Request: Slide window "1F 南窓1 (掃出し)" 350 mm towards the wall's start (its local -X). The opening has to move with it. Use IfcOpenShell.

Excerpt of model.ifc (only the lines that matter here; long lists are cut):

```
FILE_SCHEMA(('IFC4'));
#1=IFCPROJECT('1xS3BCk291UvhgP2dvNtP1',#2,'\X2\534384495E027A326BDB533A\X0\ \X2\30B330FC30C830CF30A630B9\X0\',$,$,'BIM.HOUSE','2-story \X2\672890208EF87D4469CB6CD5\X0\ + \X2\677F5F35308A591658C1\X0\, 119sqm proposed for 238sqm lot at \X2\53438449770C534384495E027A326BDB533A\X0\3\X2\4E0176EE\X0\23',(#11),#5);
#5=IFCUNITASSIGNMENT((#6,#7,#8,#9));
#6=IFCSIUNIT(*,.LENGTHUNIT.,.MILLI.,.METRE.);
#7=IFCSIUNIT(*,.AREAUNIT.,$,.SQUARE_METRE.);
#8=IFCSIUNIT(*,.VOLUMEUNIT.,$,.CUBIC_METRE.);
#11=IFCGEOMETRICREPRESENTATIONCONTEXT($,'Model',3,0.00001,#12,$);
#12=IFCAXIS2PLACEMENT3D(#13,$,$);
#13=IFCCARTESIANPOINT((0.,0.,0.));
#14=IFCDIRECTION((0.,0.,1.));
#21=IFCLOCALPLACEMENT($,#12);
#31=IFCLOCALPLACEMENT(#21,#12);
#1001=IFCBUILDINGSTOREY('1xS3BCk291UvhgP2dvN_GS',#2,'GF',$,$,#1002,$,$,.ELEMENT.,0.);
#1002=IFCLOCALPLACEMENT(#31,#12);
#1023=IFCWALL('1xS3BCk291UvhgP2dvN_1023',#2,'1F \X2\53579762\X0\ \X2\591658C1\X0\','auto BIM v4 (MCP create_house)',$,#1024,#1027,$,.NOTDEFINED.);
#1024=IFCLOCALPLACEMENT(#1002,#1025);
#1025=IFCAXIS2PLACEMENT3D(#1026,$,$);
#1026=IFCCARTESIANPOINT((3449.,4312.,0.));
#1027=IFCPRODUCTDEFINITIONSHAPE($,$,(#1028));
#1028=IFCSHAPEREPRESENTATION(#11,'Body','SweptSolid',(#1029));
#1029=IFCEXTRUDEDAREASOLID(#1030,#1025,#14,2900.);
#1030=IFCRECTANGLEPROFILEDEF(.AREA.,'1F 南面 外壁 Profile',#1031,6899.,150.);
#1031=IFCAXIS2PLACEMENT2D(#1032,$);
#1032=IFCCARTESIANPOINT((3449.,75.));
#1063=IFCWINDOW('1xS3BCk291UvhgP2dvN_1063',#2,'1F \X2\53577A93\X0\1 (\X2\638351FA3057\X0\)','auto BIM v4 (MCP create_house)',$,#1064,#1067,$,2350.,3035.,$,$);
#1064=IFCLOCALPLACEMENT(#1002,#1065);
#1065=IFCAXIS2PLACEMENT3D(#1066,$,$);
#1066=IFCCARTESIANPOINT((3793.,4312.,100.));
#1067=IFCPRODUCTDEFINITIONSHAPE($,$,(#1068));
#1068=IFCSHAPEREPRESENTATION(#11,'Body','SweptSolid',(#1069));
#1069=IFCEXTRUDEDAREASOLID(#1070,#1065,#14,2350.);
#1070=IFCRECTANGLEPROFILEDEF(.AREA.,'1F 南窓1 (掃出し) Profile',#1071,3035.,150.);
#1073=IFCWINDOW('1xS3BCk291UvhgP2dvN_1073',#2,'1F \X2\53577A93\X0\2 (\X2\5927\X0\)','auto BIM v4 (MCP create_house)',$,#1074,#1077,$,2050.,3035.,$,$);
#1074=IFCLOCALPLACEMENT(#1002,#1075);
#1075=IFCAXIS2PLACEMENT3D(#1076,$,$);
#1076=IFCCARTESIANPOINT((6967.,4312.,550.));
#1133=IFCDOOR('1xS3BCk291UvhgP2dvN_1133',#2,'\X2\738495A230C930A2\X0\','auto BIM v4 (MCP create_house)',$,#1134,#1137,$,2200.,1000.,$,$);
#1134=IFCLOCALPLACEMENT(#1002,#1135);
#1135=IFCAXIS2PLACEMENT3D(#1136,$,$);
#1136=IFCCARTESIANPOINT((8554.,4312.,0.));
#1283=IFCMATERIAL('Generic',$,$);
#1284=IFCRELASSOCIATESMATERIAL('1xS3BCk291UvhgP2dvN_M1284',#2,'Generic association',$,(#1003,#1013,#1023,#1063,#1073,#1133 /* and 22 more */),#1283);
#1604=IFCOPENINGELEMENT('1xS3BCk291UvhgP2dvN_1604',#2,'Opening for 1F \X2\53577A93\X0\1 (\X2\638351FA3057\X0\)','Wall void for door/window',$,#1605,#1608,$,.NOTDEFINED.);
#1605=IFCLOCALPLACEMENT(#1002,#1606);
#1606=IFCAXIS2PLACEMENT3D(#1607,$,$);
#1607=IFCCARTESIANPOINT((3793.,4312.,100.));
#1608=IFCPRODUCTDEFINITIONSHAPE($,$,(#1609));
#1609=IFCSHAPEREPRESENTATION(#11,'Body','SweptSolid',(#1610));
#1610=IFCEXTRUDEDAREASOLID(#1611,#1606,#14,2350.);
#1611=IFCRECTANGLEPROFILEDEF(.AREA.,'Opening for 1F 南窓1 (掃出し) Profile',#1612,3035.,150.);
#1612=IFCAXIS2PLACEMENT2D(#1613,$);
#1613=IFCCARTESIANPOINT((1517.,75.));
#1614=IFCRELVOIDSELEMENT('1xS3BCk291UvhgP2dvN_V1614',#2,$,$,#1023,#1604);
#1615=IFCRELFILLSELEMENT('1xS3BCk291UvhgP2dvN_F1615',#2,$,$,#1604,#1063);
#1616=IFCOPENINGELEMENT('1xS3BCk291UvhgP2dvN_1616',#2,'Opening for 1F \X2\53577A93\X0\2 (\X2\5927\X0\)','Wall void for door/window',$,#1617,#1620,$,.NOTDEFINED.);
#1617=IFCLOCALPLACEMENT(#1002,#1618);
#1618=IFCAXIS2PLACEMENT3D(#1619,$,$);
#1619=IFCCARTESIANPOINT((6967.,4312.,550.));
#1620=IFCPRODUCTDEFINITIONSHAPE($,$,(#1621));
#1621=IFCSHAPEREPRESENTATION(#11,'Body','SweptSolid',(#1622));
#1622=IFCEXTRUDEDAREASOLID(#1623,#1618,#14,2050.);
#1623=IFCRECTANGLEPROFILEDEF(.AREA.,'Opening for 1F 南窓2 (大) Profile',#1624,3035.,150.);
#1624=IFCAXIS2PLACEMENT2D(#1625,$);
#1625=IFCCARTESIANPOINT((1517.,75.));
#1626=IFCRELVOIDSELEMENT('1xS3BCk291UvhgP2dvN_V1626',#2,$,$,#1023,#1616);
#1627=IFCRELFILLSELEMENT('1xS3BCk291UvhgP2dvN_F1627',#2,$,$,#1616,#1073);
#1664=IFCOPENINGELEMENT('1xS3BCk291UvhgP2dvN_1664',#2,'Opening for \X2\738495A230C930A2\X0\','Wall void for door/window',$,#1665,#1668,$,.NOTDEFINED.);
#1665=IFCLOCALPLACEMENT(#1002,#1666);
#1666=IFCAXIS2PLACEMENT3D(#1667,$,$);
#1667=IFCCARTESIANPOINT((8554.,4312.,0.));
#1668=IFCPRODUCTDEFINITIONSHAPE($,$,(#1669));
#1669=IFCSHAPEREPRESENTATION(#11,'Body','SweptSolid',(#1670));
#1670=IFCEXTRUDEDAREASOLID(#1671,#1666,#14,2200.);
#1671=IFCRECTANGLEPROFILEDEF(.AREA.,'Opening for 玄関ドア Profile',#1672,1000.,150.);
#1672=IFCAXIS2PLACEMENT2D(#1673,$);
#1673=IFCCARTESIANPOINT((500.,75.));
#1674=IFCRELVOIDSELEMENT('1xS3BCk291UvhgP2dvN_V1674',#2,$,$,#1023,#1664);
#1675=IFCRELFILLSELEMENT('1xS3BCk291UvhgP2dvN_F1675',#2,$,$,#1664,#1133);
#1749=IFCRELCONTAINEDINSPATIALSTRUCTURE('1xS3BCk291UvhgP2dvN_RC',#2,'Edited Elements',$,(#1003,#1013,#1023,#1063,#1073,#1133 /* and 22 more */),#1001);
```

```python
import ifcopenshell
import ifcopenshell.api.geometry
import ifcopenshell.util.placement

model = ifcopenshell.open("model.ifc")

window = model.by_id(1063)
opening = window.FillsVoids[0].RelatingOpeningElement
wall = opening.VoidsElements[0].RelatingBuildingElement

wall_matrix = ifcopenshell.util.placement.get_local_placement(wall.ObjectPlacement)
shift = wall_matrix[:3, 0] * -350.0
before = ifcopenshell.util.placement.get_local_placement(window.ObjectPlacement)[:3, 3].copy()

# The window is not placed relative to its opening, so move both.
for product in (opening, window):
    matrix = ifcopenshell.util.placement.get_local_placement(product.ObjectPlacement)
    matrix[:3, 3] += shift
    ifcopenshell.api.geometry.edit_object_placement(model, product=product, matrix=matrix, is_si=False)

after = ifcopenshell.util.placement.get_local_placement(window.ObjectPlacement)[:3, 3]
print("window moved by", (after - before).round(3) + 0.0)

model.write("model_v2.ifc")
```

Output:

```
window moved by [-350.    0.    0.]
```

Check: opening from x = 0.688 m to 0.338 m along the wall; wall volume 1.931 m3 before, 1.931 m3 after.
